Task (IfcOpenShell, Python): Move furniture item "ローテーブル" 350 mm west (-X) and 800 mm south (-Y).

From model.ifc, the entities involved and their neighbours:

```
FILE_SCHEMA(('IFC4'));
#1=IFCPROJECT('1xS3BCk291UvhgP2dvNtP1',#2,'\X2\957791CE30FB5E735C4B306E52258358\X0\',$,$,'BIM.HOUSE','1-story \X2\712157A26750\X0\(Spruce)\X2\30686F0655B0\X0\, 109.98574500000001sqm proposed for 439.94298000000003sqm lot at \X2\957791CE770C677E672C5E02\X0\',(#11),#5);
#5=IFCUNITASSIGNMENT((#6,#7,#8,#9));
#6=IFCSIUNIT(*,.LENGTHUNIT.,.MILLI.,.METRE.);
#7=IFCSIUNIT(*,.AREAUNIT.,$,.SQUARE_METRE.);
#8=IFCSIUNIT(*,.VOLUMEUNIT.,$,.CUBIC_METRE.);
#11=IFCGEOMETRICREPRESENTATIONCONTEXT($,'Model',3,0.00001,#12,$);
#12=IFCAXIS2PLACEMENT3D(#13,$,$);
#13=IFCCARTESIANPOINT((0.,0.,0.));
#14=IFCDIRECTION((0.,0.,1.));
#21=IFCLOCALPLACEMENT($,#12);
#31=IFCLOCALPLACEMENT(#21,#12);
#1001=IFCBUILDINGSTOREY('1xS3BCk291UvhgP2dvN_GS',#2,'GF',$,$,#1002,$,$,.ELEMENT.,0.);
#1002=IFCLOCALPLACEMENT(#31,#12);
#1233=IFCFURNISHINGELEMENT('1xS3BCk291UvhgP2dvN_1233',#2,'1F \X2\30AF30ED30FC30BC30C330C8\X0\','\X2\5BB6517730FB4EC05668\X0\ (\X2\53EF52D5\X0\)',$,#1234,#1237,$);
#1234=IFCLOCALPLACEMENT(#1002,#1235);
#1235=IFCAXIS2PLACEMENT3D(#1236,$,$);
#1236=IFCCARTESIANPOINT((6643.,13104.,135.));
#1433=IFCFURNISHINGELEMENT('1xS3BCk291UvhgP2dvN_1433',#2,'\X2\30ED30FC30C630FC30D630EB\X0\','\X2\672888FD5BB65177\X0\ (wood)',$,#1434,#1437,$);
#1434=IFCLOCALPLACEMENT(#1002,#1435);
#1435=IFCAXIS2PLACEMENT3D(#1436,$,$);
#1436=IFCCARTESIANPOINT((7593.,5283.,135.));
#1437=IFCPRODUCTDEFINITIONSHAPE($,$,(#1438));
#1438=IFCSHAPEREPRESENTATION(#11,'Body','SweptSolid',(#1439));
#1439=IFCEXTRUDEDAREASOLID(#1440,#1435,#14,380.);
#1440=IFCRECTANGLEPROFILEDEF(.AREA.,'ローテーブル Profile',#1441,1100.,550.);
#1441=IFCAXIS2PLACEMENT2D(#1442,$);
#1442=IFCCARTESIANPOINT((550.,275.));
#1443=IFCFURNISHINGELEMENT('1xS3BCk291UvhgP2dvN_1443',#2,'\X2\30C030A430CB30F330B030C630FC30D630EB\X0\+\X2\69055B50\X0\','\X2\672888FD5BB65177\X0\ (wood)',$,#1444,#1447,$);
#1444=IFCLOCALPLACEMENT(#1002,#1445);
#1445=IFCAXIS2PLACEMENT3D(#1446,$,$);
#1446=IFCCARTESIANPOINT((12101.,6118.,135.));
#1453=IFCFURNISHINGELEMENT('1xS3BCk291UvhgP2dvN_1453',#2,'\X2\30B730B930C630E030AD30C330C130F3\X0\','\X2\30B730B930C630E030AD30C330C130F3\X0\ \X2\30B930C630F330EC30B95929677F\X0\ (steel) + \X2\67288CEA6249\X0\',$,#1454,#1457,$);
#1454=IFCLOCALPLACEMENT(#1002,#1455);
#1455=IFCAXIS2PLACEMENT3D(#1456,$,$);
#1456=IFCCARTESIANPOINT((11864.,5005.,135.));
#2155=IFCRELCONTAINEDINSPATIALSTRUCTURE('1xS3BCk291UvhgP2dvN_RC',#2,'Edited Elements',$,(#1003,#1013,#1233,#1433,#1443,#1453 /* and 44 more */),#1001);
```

```python
import ifcopenshell
import ifcopenshell.api.geometry
import ifcopenshell.util.placement
import ifcopenshell.util.unit

model = ifcopenshell.open("model.ifc")
unit_scale = ifcopenshell.util.unit.calculate_unit_scale(model)

item = model.by_guid("1xS3BCk291UvhgP2dvN_1433")
matrix = ifcopenshell.util.placement.get_local_placement(item.ObjectPlacement)
matrix[0, 3] -= 0.35 / unit_scale
matrix[1, 3] -= 0.8 / unit_scale
ifcopenshell.api.geometry.edit_object_placement(model, product=item, matrix=matrix, is_si=False)

print(ifcopenshell.util.placement.get_local_placement(item.ObjectPlacement).round(3) + 0.0)

model.write("model_updated.ifc")
```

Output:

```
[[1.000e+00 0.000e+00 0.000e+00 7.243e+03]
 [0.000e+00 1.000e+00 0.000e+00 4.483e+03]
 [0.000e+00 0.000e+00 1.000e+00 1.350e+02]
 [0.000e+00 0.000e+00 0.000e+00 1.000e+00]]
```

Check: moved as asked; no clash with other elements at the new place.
